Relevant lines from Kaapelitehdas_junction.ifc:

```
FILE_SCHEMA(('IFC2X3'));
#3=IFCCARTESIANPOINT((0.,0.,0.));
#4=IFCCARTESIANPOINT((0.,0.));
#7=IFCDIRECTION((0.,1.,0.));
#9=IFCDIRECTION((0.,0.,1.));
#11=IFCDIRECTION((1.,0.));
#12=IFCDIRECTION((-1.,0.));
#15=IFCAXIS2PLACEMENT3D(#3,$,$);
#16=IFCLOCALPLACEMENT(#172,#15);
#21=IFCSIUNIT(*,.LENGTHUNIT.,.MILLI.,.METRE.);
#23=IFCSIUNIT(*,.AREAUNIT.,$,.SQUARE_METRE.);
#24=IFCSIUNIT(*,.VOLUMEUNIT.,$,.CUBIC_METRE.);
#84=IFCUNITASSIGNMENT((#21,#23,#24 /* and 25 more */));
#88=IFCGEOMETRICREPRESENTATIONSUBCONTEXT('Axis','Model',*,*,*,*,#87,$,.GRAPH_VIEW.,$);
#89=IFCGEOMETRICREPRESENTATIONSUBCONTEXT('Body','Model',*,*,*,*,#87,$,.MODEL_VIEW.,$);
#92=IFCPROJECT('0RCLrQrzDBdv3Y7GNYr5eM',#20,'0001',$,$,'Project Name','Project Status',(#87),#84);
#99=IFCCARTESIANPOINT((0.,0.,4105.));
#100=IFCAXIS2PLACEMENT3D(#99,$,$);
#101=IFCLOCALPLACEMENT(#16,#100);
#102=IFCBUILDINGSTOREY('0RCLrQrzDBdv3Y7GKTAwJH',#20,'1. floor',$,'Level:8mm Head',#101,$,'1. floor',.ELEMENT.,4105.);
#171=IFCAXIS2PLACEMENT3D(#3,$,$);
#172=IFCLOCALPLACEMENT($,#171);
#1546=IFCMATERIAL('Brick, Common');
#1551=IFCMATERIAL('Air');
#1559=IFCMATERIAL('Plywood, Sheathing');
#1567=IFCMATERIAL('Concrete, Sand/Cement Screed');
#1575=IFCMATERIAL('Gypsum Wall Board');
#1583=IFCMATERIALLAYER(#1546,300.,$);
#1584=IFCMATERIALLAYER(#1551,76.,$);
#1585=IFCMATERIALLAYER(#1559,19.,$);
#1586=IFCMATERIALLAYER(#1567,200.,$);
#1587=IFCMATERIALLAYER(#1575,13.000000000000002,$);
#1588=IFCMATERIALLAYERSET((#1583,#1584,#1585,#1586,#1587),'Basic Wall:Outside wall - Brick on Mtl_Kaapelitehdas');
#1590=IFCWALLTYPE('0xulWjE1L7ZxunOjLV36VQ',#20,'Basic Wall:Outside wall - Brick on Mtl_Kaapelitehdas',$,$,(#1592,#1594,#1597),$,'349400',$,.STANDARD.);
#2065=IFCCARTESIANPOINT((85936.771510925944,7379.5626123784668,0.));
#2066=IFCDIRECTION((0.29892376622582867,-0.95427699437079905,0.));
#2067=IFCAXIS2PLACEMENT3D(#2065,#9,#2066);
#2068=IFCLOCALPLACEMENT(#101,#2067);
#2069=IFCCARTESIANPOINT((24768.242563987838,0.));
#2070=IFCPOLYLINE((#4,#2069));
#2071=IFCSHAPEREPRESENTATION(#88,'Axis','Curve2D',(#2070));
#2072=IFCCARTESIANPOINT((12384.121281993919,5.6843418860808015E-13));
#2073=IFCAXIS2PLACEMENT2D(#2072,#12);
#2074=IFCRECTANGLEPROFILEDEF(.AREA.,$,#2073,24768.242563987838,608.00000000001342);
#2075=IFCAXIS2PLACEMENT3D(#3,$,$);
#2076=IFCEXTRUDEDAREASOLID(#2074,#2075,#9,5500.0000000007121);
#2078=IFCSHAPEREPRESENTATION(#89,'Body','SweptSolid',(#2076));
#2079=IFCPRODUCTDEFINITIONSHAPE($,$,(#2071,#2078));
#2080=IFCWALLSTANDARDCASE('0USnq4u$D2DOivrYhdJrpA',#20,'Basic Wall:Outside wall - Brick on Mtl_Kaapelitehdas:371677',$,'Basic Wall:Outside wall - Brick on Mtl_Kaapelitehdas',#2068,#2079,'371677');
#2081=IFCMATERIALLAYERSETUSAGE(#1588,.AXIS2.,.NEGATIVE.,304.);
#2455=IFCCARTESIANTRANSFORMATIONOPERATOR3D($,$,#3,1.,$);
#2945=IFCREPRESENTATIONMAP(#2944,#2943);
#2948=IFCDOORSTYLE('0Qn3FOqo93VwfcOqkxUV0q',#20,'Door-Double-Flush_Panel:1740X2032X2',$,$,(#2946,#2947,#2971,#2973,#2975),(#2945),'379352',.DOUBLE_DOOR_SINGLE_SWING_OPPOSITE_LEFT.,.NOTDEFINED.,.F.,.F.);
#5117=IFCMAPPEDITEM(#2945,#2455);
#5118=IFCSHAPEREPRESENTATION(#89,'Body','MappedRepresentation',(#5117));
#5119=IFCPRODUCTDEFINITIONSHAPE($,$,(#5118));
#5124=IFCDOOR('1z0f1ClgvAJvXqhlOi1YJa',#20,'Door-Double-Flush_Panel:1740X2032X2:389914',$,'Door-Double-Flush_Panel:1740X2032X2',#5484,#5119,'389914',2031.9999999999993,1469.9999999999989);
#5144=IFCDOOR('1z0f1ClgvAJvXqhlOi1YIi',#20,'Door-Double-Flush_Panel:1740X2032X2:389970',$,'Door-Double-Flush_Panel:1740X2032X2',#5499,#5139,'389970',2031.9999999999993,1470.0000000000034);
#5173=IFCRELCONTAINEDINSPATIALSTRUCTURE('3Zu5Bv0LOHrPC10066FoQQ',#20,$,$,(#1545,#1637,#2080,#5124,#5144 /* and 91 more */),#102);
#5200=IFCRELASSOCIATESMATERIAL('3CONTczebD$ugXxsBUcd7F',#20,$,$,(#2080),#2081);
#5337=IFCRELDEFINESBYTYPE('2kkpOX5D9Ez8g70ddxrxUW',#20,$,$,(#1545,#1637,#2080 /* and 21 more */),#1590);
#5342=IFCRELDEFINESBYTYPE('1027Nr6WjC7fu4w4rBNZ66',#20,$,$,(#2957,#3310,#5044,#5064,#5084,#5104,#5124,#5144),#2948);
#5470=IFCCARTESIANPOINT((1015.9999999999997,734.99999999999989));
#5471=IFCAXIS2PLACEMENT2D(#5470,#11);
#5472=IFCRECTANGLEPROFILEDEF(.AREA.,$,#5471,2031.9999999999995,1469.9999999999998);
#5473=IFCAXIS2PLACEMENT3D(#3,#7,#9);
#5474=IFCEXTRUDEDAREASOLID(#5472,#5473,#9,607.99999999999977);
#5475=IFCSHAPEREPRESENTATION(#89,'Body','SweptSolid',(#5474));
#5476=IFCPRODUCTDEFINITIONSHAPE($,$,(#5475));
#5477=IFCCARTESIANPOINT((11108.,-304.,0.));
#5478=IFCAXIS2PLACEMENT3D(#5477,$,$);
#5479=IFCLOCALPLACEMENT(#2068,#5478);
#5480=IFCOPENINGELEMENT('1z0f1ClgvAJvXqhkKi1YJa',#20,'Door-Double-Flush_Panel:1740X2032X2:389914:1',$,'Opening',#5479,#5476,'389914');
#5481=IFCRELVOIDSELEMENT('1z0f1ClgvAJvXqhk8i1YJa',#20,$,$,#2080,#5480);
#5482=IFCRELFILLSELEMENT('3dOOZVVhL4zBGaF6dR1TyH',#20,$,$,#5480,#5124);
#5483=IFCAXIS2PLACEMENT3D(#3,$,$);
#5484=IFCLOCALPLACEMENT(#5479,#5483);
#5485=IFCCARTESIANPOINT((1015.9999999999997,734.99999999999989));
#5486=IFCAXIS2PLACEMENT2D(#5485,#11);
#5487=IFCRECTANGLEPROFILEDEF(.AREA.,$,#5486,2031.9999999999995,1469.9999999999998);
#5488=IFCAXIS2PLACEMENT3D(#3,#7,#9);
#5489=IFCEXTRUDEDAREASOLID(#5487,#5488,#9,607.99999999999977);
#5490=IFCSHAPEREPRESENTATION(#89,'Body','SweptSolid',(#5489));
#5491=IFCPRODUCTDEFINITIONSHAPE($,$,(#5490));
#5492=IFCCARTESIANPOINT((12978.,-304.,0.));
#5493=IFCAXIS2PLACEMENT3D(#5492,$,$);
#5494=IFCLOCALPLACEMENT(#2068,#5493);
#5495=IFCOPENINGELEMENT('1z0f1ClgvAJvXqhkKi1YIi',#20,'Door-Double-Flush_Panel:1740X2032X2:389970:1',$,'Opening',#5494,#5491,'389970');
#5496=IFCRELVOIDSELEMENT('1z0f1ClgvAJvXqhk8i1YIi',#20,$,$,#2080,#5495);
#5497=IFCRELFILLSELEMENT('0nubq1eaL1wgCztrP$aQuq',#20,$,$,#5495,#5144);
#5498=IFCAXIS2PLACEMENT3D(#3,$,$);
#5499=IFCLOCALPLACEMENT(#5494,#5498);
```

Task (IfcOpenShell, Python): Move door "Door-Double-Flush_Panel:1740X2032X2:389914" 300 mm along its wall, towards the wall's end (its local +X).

```python
import ifcopenshell
import ifcopenshell.api.geometry
import ifcopenshell.util.placement

model = ifcopenshell.open("Kaapelitehdas_junction.ifc")

door = model.by_id(5124)
opening = door.FillsVoids[0].RelatingOpeningElement
wall = opening.VoidsElements[0].RelatingBuildingElement

wall_matrix = ifcopenshell.util.placement.get_local_placement(wall.ObjectPlacement)
shift = wall_matrix[:3, 0] * 300.0
before = ifcopenshell.util.placement.get_local_placement(door.ObjectPlacement)[:3, 3].copy()

# The door is placed relative to its opening, so it follows when the opening moves.
matrix = ifcopenshell.util.placement.get_local_placement(opening.ObjectPlacement)
matrix[:3, 3] += shift
ifcopenshell.api.geometry.edit_object_placement(
    model, product=opening, matrix=matrix, is_si=False, should_transform_children=True
)

after = ifcopenshell.util.placement.get_local_placement(door.ObjectPlacement)[:3, 3]
print("door moved by", (after - before).round(3) + 0.0)

model.write("Kaapelitehdas_junction_v2.ifc")
```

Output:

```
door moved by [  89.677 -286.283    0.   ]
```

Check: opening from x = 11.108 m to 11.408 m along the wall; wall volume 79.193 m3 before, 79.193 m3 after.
